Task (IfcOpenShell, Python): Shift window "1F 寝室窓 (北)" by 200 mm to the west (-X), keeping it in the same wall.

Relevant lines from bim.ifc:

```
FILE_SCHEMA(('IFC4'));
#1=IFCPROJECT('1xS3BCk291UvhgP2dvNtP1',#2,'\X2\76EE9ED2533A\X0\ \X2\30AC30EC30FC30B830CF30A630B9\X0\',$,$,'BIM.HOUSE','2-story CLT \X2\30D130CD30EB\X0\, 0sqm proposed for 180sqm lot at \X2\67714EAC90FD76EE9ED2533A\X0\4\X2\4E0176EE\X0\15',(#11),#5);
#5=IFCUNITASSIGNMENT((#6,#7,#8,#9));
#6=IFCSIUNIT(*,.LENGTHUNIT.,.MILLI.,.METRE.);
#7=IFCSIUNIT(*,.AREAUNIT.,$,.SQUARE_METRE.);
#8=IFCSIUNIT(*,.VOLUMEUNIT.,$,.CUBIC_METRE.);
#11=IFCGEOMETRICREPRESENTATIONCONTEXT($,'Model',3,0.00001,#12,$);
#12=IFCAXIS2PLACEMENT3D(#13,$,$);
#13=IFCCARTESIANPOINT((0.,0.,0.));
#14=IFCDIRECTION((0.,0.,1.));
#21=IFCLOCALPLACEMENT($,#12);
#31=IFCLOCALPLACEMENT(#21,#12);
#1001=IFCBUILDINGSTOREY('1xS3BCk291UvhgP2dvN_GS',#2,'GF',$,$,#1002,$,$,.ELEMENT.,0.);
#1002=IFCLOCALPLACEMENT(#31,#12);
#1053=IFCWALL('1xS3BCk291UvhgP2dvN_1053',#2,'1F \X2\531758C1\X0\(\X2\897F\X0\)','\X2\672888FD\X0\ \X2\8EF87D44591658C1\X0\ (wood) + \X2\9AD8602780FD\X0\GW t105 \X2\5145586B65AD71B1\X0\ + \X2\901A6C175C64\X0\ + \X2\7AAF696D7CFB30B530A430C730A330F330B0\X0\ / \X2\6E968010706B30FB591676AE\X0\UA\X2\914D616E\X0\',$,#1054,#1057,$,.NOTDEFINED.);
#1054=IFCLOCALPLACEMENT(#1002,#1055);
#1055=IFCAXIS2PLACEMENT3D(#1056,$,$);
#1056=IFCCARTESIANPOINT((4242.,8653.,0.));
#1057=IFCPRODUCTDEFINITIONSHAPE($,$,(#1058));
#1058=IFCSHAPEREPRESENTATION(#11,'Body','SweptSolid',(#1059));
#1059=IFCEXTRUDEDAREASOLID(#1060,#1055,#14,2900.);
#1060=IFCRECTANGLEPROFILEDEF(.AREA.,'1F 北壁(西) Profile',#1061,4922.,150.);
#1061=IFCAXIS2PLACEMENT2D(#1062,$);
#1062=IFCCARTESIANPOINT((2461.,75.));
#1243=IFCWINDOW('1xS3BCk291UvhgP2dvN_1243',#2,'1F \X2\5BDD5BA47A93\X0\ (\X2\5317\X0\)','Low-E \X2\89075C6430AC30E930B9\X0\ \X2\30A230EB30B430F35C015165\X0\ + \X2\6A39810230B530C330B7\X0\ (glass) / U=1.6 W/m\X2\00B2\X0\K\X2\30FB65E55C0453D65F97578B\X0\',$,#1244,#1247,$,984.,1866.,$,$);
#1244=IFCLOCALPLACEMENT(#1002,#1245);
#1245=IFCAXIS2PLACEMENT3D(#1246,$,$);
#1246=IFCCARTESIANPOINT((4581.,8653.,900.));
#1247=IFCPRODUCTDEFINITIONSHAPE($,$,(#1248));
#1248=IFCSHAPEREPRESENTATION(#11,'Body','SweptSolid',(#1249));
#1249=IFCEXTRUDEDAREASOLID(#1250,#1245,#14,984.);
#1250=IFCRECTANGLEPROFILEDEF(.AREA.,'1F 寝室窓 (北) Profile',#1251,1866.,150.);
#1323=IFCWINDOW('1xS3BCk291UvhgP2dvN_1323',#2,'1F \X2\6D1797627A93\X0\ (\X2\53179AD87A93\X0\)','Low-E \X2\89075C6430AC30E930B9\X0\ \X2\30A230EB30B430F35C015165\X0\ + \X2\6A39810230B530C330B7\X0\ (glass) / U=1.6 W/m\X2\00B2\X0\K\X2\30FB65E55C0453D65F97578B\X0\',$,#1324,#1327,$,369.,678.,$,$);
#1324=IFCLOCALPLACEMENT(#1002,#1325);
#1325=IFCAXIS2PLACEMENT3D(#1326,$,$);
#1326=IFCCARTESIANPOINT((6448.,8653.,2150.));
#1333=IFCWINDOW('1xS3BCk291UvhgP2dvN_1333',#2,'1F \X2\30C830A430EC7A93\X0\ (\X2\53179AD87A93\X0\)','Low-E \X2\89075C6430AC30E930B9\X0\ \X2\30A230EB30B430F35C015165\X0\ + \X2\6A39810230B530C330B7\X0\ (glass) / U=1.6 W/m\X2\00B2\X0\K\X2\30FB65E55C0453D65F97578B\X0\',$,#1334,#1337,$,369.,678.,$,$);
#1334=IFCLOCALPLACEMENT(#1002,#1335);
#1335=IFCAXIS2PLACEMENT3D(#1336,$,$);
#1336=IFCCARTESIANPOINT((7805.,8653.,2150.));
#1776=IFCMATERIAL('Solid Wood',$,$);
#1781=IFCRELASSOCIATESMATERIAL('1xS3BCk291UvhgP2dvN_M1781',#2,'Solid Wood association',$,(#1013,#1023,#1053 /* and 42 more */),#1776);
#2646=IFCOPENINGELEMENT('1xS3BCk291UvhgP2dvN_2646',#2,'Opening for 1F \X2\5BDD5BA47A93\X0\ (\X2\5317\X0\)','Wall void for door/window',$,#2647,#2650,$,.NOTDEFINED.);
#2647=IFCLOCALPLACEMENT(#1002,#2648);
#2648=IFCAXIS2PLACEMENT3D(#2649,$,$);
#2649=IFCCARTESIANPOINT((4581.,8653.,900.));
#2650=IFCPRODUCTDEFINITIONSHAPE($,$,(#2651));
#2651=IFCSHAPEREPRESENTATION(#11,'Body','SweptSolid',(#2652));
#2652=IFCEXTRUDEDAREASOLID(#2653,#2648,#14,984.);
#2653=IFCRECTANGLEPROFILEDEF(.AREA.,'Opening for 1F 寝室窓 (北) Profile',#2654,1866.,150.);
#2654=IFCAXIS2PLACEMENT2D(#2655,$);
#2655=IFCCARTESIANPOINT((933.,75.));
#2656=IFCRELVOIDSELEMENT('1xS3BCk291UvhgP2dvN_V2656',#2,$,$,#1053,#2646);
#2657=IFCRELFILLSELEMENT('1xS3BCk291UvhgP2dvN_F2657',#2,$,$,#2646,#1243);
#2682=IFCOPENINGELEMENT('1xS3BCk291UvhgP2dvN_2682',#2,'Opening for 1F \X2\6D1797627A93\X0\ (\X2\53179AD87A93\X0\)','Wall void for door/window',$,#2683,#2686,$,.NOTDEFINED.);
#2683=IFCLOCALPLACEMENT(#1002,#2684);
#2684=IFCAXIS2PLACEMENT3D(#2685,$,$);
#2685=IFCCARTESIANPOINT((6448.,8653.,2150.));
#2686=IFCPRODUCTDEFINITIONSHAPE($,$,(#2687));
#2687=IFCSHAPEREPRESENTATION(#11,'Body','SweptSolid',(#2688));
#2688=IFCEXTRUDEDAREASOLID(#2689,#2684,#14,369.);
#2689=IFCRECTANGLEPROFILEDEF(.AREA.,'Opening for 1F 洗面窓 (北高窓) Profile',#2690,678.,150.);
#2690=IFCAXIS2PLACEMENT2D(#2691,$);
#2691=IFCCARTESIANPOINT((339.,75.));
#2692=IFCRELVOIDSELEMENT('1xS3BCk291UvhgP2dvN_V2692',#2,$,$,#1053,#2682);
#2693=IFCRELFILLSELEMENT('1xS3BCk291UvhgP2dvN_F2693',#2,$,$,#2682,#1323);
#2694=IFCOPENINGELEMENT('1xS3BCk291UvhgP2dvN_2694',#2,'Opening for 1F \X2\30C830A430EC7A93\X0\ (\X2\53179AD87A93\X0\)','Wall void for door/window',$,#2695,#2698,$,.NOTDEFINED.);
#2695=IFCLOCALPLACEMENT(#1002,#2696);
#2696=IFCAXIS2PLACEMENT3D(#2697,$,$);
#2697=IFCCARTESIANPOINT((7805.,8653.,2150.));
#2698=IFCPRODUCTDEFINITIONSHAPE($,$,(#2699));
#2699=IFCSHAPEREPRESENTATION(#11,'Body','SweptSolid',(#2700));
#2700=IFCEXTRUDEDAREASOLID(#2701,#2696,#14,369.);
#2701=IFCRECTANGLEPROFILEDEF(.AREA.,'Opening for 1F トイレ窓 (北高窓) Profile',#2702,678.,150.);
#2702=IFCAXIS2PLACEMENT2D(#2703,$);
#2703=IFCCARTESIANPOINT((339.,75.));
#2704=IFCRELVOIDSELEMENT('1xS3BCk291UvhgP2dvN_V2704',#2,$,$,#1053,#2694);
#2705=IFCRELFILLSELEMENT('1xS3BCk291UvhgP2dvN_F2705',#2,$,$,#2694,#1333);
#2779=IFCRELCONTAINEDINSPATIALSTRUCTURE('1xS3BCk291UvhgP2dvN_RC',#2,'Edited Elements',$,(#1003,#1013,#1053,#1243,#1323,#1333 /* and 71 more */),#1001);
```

```python
import ifcopenshell
import ifcopenshell.api.geometry
import ifcopenshell.util.placement

model = ifcopenshell.open("bim.ifc")

window = model.by_guid("1xS3BCk291UvhgP2dvN_1243")
opening = window.FillsVoids[0].RelatingOpeningElement
wall = opening.VoidsElements[0].RelatingBuildingElement

wall_matrix = ifcopenshell.util.placement.get_local_placement(wall.ObjectPlacement)
shift = wall_matrix[:3, 0] * -200.0
before = ifcopenshell.util.placement.get_local_placement(window.ObjectPlacement)[:3, 3].copy()

# The window is not placed relative to its opening, so move both.
for product in (opening, window):
    matrix = ifcopenshell.util.placement.get_local_placement(product.ObjectPlacement)
    matrix[:3, 3] += shift
    ifcopenshell.api.geometry.edit_object_placement(model, product=product, matrix=matrix, is_si=False)

after = ifcopenshell.util.placement.get_local_placement(window.ObjectPlacement)[:3, 3]
print("window moved by", (after - before).round(3) + 0.0)

model.write("bim_edited.ifc")
```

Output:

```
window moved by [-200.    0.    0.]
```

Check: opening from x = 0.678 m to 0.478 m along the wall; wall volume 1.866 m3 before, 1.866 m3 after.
